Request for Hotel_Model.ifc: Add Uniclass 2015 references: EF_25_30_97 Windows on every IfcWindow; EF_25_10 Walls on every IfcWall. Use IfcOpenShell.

First a look at what the model holds.

```python
import ifcopenshell

model = ifcopenshell.open("Hotel_Model.ifc")
print(model.schema)
print("classifications:", [c.Name for c in model.by_type("IfcClassification")])
for ifc_class in ("IfcDoor", "IfcRoof", "IfcStair", "IfcWall", "IfcWindow"):
    print(ifc_class, len(model.by_type(ifc_class)))
```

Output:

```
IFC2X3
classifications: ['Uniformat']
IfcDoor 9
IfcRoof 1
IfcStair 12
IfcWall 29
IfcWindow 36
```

```python
import ifcopenshell
import ifcopenshell.api.classification

model = ifcopenshell.open("Hotel_Model.ifc")

# IFC2X3 requires Source and Edition and has no link from the project to the system.
system = model.create_entity("IfcClassification", Source="NBS", Edition="2015", Name="Uniclass 2015")

codes = {
    "IfcWindow": ("EF_25_30_97", "Windows"),
    "IfcWall": ("EF_25_10", "Walls"),
}
for ifc_class, (code, name) in codes.items():
    products = model.by_type(ifc_class)
    ifcopenshell.api.classification.add_reference(
        model, products=products, classification=system, identification=code, name=name
    )
    print(code, len(products))

model.write("Hotel_Model_v2.ifc")
```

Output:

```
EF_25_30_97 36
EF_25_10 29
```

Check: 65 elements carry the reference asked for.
